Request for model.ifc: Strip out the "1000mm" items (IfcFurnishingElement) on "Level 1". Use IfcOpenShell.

First a look at what the model holds.

```python
import ifcopenshell
import ifcopenshell.util.element

model = ifcopenshell.open("model.ifc")
print(model.schema)
storey = next(s for s in model.by_type("IfcBuildingStorey") if s.Name == "Level 1")
furniture = [e for e in ifcopenshell.util.element.get_decomposition(storey) if e.is_a("IfcFurnishingElement")]
seen = {}
for e in furniture:
    element_type = ifcopenshell.util.element.get_type(e)
    name = element_type.Name if element_type not in (None, e) else None
    seen[name] = seen.get(name, 0) + 1
for name, count in sorted(seen.items(), key=str):
    print(count, "x", name)
```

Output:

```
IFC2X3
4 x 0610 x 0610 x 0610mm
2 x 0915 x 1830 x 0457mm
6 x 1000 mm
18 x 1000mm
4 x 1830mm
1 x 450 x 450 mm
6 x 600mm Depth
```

```python
import ifcopenshell
import ifcopenshell.api.root
import ifcopenshell.util.element

model = ifcopenshell.open("model.ifc")

storey = next(s for s in model.by_type("IfcBuildingStorey") if s.Name == "Level 1")
furniture = [e for e in ifcopenshell.util.element.get_decomposition(storey) if e.is_a("IfcFurnishingElement")]
targets = [e for e in furniture if (t := ifcopenshell.util.element.get_type(e)) not in (None, e) and t.Name == "1000mm"]

for e in targets:
    ifcopenshell.api.root.remove_product(model, product=e)
print(len(targets), "removed")

model.write("model-out.ifc")
```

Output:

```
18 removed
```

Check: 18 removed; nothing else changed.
